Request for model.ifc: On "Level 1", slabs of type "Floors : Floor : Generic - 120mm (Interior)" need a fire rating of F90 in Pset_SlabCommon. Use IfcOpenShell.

First a look at what the model holds.

```python
import ifcopenshell
import ifcopenshell.util.element

model = ifcopenshell.open("model.ifc")
print(model.schema)
storey = next(s for s in model.by_type("IfcBuildingStorey") if s.Name == "Level 1")
slabs = [e for e in ifcopenshell.util.element.get_decomposition(storey) if e.is_a("IfcSlab")]
seen = {}
for e in slabs:
    element_type = ifcopenshell.util.element.get_type(e)
    key = (element_type.Name if element_type != e and element_type else None, ifcopenshell.util.element.get_pset(e, "Pset_SlabCommon", "FireRating"))
    seen[key] = seen.get(key, 0) + 1
for (name, value), count in sorted(seen.items(), key=str):
    print(count, "x", name, "|", value)
```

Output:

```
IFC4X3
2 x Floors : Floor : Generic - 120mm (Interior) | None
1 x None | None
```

```python
import ifcopenshell
import ifcopenshell.api.pset
import ifcopenshell.util.element

model = ifcopenshell.open("model.ifc")

storey = next(s for s in model.by_type("IfcBuildingStorey") if s.Name == "Level 1")
slabs = [e for e in ifcopenshell.util.element.get_decomposition(storey) if e.is_a("IfcSlab")]

count = 0
for e in slabs:
    element_type = ifcopenshell.util.element.get_type(e)
    if element_type in (None, e) or element_type.Name != "Floors : Floor : Generic - 120mm (Interior)":
        continue
    # add_pset returns the element's existing set when there is one.
    pset = ifcopenshell.api.pset.add_pset(model, product=e, name="Pset_SlabCommon")
    ifcopenshell.api.pset.edit_pset(model, pset=pset, properties={"FireRating": "F90"})
    count += 1

print(count, "slabs updated")

model.write("model_rev.ifc")
```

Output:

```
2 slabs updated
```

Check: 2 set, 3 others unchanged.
